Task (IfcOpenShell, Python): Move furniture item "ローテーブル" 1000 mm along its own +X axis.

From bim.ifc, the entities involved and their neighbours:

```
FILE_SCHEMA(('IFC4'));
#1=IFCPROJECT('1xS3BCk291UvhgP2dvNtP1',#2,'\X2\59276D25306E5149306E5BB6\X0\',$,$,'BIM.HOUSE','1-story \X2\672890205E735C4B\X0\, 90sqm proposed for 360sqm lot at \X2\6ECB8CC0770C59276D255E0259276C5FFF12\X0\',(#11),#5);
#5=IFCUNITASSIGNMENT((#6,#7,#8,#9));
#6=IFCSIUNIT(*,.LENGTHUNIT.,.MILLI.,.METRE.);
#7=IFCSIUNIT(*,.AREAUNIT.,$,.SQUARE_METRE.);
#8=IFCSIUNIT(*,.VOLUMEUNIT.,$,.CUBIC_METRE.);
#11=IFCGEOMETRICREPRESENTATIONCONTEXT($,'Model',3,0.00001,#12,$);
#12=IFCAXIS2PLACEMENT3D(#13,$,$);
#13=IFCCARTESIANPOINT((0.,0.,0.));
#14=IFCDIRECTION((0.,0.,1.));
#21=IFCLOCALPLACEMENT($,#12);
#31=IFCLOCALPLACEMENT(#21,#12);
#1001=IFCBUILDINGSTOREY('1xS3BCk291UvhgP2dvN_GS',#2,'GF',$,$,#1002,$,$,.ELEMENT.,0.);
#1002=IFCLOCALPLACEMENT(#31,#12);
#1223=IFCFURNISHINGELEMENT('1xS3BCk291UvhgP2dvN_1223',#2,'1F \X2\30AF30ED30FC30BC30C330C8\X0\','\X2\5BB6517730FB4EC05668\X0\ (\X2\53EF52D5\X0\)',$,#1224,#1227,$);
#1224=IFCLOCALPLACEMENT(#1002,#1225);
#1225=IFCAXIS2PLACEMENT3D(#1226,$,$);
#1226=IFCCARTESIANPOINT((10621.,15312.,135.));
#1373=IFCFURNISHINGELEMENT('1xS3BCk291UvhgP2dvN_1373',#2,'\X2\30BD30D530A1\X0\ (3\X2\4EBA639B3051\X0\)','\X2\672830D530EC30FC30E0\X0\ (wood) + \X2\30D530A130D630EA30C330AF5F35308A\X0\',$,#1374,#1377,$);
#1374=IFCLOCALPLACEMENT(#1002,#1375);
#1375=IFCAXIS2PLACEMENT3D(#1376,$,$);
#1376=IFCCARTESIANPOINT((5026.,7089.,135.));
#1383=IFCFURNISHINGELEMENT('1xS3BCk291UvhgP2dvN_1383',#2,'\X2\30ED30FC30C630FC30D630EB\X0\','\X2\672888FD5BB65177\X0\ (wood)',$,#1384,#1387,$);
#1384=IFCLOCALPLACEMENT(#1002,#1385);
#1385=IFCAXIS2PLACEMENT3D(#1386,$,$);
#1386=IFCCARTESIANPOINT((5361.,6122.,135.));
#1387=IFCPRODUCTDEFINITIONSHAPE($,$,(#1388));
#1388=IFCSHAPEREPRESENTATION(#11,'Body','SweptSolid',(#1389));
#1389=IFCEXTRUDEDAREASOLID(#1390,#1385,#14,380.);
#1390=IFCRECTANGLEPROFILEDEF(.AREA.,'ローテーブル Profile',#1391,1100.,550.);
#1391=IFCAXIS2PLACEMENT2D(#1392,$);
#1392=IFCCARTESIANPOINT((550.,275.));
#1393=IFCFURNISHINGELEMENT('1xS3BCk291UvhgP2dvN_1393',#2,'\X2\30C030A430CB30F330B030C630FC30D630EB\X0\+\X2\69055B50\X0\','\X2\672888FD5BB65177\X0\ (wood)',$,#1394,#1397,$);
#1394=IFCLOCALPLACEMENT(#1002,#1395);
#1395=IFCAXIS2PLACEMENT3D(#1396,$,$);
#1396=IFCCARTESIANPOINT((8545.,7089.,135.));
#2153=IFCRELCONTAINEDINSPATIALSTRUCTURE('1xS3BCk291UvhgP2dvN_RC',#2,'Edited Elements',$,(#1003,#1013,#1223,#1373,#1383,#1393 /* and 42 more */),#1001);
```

```python
import ifcopenshell
import ifcopenshell.api.geometry
import ifcopenshell.util.placement
import ifcopenshell.util.unit

model = ifcopenshell.open("bim.ifc")
unit_scale = ifcopenshell.util.unit.calculate_unit_scale(model)

item = model.by_guid("1xS3BCk291UvhgP2dvN_1383")
matrix = ifcopenshell.util.placement.get_local_placement(item.ObjectPlacement)
matrix[:3, 3] += matrix[:3, 0] * 1 / unit_scale
ifcopenshell.api.geometry.edit_object_placement(model, product=item, matrix=matrix, is_si=False)

print(ifcopenshell.util.placement.get_local_placement(item.ObjectPlacement).round(3) + 0.0)

model.write("bim_updated.ifc")
```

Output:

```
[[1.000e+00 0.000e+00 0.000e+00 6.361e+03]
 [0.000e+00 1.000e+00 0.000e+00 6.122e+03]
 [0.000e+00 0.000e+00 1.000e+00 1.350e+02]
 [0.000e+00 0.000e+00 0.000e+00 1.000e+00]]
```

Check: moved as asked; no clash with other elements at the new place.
